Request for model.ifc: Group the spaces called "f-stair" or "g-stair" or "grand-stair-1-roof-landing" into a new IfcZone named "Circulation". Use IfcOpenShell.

First a look at what the model holds.

```python
import ifcopenshell

model = ifcopenshell.open("model.ifc")
print(model.schema)
seen = {}
for space in model.by_type("IfcSpace"):
    seen[space.LongName] = seen.get(space.LongName, 0) + 1
for name, count in sorted(seen.items(), key=str):
    print(count, "x", name)
print("zones:", [z.Name for z in model.by_type("IfcZone")][:20])
```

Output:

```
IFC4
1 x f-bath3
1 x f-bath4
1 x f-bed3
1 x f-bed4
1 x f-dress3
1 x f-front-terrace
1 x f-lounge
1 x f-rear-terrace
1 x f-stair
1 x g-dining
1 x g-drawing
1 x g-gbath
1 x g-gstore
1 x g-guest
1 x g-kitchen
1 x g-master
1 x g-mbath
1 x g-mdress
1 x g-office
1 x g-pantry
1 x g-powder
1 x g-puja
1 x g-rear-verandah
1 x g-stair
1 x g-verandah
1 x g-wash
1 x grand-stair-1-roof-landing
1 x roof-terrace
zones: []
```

```python
import ifcopenshell
import ifcopenshell.api.group
import ifcopenshell.api.root

model = ifcopenshell.open("model.ifc")

names = {"f-stair", "g-stair", "grand-stair-1-roof-landing"}
spaces = [s for s in model.by_type("IfcSpace") if s.LongName in names]

zone = ifcopenshell.api.root.create_entity(model, ifc_class="IfcZone", name="Circulation")
ifcopenshell.api.group.assign_group(model, products=spaces, group=zone)
print(len(spaces), "spaces in", zone.Name)

model.write("model_updated.ifc")
```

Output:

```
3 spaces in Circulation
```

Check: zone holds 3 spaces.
